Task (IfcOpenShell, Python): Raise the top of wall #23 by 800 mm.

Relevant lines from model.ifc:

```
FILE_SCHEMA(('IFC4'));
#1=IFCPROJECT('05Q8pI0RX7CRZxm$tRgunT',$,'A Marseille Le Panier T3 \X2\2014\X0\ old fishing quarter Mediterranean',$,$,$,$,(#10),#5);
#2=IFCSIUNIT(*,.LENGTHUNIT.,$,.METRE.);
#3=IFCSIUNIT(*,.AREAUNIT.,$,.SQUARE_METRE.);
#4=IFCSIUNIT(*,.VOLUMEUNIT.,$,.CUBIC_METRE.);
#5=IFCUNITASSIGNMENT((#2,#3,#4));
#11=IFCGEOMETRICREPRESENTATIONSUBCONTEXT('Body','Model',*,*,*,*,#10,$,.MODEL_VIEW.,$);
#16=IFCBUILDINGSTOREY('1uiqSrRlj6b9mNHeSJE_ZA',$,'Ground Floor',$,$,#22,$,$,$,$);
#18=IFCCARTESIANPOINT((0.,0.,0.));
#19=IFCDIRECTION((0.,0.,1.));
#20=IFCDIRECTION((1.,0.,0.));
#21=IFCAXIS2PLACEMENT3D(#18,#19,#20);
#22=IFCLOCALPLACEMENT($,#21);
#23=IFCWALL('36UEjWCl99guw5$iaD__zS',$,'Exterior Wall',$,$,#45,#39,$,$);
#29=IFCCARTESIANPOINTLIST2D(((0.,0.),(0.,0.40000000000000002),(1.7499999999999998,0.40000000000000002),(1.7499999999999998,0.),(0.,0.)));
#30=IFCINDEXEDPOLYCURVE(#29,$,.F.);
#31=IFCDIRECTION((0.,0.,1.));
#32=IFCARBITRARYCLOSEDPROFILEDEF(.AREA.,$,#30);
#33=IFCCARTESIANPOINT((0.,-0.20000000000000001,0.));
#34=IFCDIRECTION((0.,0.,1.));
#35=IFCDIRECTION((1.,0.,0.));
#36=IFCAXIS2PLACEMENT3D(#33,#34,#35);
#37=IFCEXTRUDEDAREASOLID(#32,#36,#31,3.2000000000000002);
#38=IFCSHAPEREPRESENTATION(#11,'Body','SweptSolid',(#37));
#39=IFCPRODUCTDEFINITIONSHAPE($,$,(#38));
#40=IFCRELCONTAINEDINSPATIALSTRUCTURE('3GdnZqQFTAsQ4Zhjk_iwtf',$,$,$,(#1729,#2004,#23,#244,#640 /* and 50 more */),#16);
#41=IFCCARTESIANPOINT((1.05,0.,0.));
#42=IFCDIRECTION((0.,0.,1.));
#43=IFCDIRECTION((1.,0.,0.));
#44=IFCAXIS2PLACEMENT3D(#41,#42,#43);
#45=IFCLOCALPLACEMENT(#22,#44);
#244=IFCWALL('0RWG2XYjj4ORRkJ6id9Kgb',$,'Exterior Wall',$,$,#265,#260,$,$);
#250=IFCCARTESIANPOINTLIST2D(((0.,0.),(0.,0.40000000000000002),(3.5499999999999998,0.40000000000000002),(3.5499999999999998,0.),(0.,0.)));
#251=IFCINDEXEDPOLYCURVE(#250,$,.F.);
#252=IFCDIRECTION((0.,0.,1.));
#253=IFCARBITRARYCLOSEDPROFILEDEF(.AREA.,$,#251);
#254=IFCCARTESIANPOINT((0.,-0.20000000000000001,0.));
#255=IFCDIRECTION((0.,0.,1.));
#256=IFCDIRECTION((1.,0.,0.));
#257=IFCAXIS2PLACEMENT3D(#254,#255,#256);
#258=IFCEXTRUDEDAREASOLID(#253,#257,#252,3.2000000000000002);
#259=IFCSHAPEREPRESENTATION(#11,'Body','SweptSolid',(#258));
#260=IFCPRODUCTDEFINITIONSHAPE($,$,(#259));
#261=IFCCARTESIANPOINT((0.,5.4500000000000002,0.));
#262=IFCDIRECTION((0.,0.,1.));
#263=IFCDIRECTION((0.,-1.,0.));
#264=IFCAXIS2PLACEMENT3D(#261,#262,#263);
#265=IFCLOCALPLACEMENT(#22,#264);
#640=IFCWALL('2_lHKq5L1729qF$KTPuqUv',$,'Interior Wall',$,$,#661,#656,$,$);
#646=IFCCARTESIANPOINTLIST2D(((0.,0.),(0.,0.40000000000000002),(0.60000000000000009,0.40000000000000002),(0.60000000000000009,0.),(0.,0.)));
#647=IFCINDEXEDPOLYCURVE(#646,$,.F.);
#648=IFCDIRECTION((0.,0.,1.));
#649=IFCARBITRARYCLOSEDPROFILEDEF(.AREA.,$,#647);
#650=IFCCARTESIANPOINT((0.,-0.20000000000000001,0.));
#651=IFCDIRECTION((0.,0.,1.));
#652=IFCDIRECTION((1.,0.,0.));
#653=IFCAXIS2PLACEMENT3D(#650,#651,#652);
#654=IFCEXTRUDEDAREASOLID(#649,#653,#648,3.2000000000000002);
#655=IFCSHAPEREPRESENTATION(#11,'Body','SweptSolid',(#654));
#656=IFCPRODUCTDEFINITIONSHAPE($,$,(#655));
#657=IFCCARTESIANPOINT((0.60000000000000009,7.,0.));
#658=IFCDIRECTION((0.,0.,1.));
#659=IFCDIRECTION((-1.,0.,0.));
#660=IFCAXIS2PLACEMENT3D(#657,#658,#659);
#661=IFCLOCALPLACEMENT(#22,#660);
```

```python
import ifcopenshell
import ifcopenshell.geom
import ifcopenshell.util.representation
import ifcopenshell.util.shape
import ifcopenshell.util.unit

model = ifcopenshell.open("model.ifc")
unit_scale = ifcopenshell.util.unit.calculate_unit_scale(model)
settings = ifcopenshell.geom.settings()


def volume(element):
    """Net volume in cubic metres, openings subtracted."""
    shape = ifcopenshell.geom.create_shape(settings, element)
    return ifcopenshell.util.shape.get_volume(shape.geometry)


wall = model.by_guid("36UEjWCl99guw5$iaD__zS")
before = volume(wall)

body = ifcopenshell.util.representation.get_representation(wall, "Model", "Body")
solid = body.Items[0]
old_height = solid.Depth
solid.Depth += 0.8 / unit_scale
after = volume(wall)

print(f"height {old_height:g} -> {solid.Depth:g}, volume {before:.3f} -> {after:.3f} m3")

model.write("model_updated.ifc")
```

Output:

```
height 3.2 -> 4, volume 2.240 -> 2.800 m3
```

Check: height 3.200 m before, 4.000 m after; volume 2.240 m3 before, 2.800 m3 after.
